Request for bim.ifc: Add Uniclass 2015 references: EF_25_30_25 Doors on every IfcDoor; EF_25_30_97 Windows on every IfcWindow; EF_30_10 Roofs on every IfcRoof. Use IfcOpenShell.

First a look at what the model holds.

```python
import ifcopenshell

model = ifcopenshell.open("bim.ifc")
print(model.schema)
print("classifications:", [c.Name for c in model.by_type("IfcClassification")])
for ifc_class in ("IfcDoor", "IfcRoof", "IfcStair", "IfcWall", "IfcWindow"):
    print(ifc_class, len(model.by_type(ifc_class)))
```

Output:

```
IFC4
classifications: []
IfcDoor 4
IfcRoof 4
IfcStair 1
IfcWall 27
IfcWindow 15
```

```python
import ifcopenshell
import ifcopenshell.api.classification

model = ifcopenshell.open("bim.ifc")

system = ifcopenshell.api.classification.add_classification(model, classification="Uniclass 2015")

codes = {
    "IfcDoor": ("EF_25_30_25", "Doors"),
    "IfcWindow": ("EF_25_30_97", "Windows"),
    "IfcRoof": ("EF_30_10", "Roofs"),
}
for ifc_class, (code, name) in codes.items():
    products = model.by_type(ifc_class)
    ifcopenshell.api.classification.add_reference(
        model, products=products, classification=system, identification=code, name=name
    )
    print(code, len(products))

model.write("bim-out.ifc")
```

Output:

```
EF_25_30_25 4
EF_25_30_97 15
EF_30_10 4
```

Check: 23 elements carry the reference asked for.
